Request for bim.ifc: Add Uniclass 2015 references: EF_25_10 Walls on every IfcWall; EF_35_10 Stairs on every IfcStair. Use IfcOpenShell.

First a look at what the model holds.

```python
import ifcopenshell

model = ifcopenshell.open("bim.ifc")
print(model.schema)
print("classifications:", [c.Name for c in model.by_type("IfcClassification")])
for ifc_class in ("IfcDoor", "IfcRoof", "IfcStair", "IfcWall", "IfcWindow"):
    print(ifc_class, len(model.by_type(ifc_class)))
```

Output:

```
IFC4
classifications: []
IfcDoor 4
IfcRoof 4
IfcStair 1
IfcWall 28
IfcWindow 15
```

```python
import ifcopenshell
import ifcopenshell.api.classification

model = ifcopenshell.open("bim.ifc")

system = ifcopenshell.api.classification.add_classification(model, classification="Uniclass 2015")

codes = {
    "IfcWall": ("EF_25_10", "Walls"),
    "IfcStair": ("EF_35_10", "Stairs"),
}
for ifc_class, (code, name) in codes.items():
    products = model.by_type(ifc_class)
    ifcopenshell.api.classification.add_reference(
        model, products=products, classification=system, identification=code, name=name
    )
    print(code, len(products))

model.write("bim_v2.ifc")
```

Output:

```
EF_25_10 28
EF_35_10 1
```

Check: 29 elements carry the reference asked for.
